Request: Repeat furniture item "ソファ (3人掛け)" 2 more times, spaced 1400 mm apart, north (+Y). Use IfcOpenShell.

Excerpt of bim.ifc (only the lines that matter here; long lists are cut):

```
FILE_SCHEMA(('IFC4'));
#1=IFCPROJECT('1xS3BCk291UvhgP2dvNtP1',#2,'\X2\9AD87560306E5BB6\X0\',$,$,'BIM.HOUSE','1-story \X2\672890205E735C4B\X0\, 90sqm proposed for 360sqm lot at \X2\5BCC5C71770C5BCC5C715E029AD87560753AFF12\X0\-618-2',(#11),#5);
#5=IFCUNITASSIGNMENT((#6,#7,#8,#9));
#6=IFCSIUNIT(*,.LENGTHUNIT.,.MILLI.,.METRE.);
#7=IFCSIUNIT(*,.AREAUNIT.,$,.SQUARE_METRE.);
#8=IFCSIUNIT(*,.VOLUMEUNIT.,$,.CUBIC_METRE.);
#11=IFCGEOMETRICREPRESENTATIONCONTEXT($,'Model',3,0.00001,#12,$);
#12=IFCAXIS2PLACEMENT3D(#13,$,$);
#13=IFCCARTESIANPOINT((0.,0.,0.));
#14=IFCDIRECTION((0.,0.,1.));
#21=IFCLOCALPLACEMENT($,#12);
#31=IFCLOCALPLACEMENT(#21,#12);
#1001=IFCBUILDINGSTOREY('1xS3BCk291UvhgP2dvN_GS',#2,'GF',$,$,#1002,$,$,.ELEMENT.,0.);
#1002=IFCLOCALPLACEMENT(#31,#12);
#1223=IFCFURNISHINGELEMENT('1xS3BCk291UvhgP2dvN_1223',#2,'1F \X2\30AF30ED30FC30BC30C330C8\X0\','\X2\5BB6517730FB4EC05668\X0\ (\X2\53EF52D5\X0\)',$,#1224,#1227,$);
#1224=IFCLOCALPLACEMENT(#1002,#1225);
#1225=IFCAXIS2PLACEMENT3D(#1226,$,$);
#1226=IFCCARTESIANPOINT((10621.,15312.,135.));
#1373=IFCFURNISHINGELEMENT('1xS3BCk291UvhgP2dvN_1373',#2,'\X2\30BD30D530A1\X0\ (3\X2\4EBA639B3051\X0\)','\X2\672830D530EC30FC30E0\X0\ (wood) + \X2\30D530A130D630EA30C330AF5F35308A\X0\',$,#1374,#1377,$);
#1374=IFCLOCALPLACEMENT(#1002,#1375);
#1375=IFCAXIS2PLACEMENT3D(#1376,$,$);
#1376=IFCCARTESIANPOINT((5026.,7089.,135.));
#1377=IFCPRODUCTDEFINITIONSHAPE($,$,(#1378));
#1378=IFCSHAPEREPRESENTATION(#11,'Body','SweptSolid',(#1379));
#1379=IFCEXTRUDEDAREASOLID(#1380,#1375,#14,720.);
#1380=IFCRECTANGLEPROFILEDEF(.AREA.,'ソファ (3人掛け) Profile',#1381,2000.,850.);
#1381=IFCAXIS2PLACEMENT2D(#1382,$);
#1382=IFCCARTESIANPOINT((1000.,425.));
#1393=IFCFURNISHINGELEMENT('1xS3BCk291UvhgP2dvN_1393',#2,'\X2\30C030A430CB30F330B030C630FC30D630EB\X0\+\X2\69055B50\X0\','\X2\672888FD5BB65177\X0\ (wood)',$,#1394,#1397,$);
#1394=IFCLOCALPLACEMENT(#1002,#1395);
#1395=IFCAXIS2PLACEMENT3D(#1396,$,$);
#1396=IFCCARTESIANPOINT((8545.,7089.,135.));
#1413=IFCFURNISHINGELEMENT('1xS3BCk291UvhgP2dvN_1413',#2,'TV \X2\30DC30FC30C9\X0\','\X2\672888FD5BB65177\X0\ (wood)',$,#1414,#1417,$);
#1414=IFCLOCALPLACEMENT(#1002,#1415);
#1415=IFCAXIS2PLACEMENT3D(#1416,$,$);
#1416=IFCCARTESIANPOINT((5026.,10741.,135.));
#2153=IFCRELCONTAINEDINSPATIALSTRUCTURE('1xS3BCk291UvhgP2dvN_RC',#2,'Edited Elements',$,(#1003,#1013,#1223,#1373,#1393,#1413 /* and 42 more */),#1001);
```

```python
import numpy as np
import ifcopenshell
import ifcopenshell.api.geometry
import ifcopenshell.api.root
import ifcopenshell.util.element
import ifcopenshell.util.placement
import ifcopenshell.util.unit

model = ifcopenshell.open("bim.ifc")
unit_scale = ifcopenshell.util.unit.calculate_unit_scale(model)


def reuse_history(source, copy):
    """copy_class also copies each property set's owner history, people and application; keep the originals."""
    for rel in copy.IsDefinedBy:
        if rel.is_a("IfcRelDefinesByProperties") and (history := rel.RelatingPropertyDefinition.OwnerHistory):
            rel.RelatingPropertyDefinition.OwnerHistory = source.OwnerHistory
            ifcopenshell.util.element.remove_deep2(model, history)


source = model.by_guid("1xS3BCk291UvhgP2dvN_1373")
base = ifcopenshell.util.placement.get_local_placement(source.ObjectPlacement)
step = np.array([0.0, 1.0, 0.0]) * 1.4 / unit_scale

for i in range(1, 3):
    copy = ifcopenshell.api.root.copy_class(model, product=source)
    copy.Representation = ifcopenshell.util.element.copy_deep(
        model, source.Representation, exclude=["IfcGeometricRepresentationContext", "IfcRepresentationMap"]
    )
    reuse_history(source, copy)
    matrix = base.copy()
    matrix[:3, 3] += i * step
    print("added at", matrix[:3, 3].round(3) + 0.0)
    ifcopenshell.api.geometry.edit_object_placement(model, product=copy, matrix=matrix, is_si=False)

model.write("bim_v2.ifc")
```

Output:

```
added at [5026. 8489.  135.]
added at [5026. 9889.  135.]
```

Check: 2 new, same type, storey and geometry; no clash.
